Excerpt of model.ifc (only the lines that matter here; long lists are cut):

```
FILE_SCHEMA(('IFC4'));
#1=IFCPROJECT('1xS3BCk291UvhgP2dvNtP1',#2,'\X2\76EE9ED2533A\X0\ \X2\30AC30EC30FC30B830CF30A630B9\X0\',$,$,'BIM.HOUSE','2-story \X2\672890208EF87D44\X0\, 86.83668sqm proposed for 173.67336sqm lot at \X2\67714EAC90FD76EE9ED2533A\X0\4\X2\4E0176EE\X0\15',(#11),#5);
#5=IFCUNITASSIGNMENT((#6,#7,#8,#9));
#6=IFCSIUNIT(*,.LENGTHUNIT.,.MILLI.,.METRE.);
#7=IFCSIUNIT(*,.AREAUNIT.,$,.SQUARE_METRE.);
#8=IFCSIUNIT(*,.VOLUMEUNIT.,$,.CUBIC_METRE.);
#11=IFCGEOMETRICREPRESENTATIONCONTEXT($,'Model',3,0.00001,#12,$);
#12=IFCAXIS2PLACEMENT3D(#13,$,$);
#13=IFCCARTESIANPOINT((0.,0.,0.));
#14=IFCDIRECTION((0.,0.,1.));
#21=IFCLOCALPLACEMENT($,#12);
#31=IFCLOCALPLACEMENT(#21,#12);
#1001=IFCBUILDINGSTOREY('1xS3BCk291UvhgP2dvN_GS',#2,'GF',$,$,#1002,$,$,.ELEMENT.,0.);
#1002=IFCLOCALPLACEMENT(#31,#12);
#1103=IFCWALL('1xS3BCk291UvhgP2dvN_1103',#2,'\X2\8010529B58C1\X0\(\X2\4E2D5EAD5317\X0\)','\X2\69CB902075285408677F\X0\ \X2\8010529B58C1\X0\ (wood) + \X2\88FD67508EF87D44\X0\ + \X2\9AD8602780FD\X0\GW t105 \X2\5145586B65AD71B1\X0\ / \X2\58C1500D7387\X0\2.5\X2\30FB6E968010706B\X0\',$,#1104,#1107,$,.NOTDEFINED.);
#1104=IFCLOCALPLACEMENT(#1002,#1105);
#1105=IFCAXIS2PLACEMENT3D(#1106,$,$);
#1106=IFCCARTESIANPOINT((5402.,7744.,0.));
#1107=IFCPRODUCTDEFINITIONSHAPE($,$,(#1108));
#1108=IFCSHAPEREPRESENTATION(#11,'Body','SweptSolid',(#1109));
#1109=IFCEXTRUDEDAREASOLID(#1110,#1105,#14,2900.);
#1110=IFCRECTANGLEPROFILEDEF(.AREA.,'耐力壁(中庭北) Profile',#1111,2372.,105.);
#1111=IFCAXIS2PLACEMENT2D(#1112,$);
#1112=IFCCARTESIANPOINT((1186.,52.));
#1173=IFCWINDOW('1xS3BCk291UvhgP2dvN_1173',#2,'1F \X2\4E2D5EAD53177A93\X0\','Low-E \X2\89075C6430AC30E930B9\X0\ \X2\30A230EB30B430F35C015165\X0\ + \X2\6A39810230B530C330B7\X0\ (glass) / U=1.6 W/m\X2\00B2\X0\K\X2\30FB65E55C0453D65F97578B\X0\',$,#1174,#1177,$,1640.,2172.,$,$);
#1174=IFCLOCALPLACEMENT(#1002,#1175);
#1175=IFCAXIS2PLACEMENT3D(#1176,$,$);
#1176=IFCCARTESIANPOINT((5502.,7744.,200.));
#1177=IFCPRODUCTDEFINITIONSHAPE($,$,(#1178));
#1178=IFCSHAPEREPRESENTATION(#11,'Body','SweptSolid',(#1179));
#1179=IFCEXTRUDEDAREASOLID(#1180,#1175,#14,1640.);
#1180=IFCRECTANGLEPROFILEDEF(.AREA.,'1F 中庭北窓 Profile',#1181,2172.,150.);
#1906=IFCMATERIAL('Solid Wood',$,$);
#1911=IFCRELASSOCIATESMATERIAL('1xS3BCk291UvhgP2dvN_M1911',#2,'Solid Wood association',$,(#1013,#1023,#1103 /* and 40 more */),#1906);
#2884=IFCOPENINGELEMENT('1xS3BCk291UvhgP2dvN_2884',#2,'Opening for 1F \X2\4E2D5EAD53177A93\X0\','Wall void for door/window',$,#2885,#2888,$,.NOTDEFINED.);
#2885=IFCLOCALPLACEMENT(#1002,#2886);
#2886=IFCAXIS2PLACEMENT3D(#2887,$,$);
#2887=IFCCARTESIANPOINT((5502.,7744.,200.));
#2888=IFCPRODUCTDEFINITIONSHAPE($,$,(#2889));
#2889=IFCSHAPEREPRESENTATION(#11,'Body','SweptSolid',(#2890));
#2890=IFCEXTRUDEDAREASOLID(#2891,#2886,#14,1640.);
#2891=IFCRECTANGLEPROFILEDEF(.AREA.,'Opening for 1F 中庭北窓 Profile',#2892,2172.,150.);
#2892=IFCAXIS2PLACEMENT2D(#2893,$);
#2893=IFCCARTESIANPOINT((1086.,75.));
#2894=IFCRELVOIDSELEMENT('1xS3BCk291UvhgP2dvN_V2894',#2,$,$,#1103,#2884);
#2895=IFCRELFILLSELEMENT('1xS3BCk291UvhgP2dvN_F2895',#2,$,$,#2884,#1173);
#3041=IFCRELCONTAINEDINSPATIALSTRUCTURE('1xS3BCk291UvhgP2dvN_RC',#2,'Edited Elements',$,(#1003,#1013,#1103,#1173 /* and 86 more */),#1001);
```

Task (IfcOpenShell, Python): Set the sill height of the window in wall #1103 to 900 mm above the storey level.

```python
import numpy as np
import ifcopenshell
import ifcopenshell.api.geometry
import ifcopenshell.geom
import ifcopenshell.util.element
import ifcopenshell.util.placement
import ifcopenshell.util.shape
import ifcopenshell.util.unit

model = ifcopenshell.open("model.ifc")
unit_scale = ifcopenshell.util.unit.calculate_unit_scale(model)

window = model.by_guid("1xS3BCk291UvhgP2dvN_1173")
opening = window.FillsVoids[0].RelatingOpeningElement
storey = ifcopenshell.util.element.get_container(window, ifc_class="IfcBuildingStorey")
level = ifcopenshell.util.placement.get_local_placement(storey.ObjectPlacement)[2, 3]

# The opening's origin need not be at the sill, so measure its lowest point.
shape = ifcopenshell.geom.create_shape(ifcopenshell.geom.settings(), opening)
bottom = ifcopenshell.util.shape.get_shape_bottom_elevation(shape, shape.geometry) / unit_scale
dz = level + 0.9 / unit_scale - bottom

shift = np.array([0.0, 0.0, dz])
# The window is not placed relative to its opening, so move both.
for product in (opening, window):
    matrix = ifcopenshell.util.placement.get_local_placement(product.ObjectPlacement)
    matrix[:3, 3] += shift
    ifcopenshell.api.geometry.edit_object_placement(model, product=product, matrix=matrix, is_si=False)

print(f"moved by {dz * unit_scale:+.3f} m")

model.write("model_edited.ifc")
```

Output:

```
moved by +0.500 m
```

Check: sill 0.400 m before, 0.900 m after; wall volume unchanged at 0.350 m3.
